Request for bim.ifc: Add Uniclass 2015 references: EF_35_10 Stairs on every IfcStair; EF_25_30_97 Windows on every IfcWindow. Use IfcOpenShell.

First a look at what the model holds.

```python
import ifcopenshell

model = ifcopenshell.open("bim.ifc")
print(model.schema)
print("classifications:", [c.Name for c in model.by_type("IfcClassification")])
for ifc_class in ("IfcDoor", "IfcRoof", "IfcStair", "IfcWall", "IfcWindow"):
    print(ifc_class, len(model.by_type(ifc_class)))
```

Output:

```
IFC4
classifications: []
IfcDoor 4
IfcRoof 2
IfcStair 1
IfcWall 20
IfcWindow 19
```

```python
import ifcopenshell
import ifcopenshell.api.classification

model = ifcopenshell.open("bim.ifc")

system = ifcopenshell.api.classification.add_classification(model, classification="Uniclass 2015")

codes = {
    "IfcStair": ("EF_35_10", "Stairs"),
    "IfcWindow": ("EF_25_30_97", "Windows"),
}
for ifc_class, (code, name) in codes.items():
    products = model.by_type(ifc_class)
    ifcopenshell.api.classification.add_reference(
        model, products=products, classification=system, identification=code, name=name
    )
    print(code, len(products))

model.write("bim_updated.ifc")
```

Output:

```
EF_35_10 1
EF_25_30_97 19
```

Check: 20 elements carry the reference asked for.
